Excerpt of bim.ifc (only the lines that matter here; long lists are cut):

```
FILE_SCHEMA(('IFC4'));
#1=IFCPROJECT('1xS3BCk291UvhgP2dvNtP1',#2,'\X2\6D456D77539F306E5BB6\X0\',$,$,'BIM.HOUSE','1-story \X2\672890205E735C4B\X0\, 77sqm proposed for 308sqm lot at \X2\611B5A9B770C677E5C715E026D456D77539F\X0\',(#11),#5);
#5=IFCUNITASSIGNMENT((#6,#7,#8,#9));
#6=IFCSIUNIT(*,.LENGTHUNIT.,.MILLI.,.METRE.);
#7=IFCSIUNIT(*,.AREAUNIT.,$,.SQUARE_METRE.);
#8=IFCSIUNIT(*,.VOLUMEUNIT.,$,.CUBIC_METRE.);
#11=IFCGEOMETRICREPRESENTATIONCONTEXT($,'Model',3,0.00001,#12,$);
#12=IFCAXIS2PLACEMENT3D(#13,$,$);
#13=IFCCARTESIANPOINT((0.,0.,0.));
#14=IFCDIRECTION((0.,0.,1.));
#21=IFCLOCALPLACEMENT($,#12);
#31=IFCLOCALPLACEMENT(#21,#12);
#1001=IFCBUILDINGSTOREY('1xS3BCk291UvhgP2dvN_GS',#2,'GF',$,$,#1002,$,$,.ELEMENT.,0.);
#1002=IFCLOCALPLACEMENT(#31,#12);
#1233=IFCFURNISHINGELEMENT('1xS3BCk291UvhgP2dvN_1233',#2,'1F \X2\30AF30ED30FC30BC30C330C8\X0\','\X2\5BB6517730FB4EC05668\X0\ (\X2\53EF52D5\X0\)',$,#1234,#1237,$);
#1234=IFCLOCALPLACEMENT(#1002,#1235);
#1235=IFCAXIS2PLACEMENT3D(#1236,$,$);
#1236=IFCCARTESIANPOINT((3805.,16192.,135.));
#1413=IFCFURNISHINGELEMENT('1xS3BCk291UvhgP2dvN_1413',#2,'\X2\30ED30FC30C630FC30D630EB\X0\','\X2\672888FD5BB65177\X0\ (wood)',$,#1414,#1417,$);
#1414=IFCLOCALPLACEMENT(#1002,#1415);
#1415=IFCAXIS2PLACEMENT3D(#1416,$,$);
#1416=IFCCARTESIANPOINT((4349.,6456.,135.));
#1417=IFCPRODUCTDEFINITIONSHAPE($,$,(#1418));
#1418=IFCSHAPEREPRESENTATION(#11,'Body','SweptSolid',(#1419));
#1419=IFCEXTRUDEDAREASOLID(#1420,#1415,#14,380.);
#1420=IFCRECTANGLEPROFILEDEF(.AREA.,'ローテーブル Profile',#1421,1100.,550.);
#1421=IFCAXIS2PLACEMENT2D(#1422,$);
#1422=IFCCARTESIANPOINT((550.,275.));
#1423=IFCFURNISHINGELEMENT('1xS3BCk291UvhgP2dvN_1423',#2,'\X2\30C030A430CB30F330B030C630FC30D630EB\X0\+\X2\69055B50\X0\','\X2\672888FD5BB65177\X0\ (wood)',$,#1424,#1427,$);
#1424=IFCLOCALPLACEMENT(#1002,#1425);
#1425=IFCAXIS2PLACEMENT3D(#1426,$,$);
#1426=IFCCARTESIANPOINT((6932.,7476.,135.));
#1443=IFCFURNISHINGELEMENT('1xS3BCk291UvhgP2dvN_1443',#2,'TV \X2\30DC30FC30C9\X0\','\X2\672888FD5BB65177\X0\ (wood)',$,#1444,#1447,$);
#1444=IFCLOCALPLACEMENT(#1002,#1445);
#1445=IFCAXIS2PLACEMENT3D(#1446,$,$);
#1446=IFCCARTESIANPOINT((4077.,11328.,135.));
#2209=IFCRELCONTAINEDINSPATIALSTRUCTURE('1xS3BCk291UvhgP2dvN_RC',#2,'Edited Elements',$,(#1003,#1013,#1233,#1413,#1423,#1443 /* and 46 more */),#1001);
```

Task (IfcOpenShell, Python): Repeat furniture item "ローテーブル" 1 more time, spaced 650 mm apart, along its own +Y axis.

```python
import ifcopenshell
import ifcopenshell.api.geometry
import ifcopenshell.api.root
import ifcopenshell.util.element
import ifcopenshell.util.placement

model = ifcopenshell.open("bim.ifc")


def reuse_history(source, copy):
    """copy_class also copies each property set's owner history, people and application; keep the originals."""
    for rel in copy.IsDefinedBy:
        if rel.is_a("IfcRelDefinesByProperties") and (history := rel.RelatingPropertyDefinition.OwnerHistory):
            rel.RelatingPropertyDefinition.OwnerHistory = source.OwnerHistory
            ifcopenshell.util.element.remove_deep2(model, history)


source = model.by_guid("1xS3BCk291UvhgP2dvN_1413")
base = ifcopenshell.util.placement.get_local_placement(source.ObjectPlacement)
step = base[:3, 1] * 650.0

for i in range(1, 2):
    copy = ifcopenshell.api.root.copy_class(model, product=source)
    copy.Representation = ifcopenshell.util.element.copy_deep(
        model, source.Representation, exclude=["IfcGeometricRepresentationContext", "IfcRepresentationMap"]
    )
    reuse_history(source, copy)
    matrix = base.copy()
    matrix[:3, 3] += i * step
    print("added at", matrix[:3, 3].round(3) + 0.0)
    ifcopenshell.api.geometry.edit_object_placement(model, product=copy, matrix=matrix, is_si=False)

model.write("bim_v2.ifc")
```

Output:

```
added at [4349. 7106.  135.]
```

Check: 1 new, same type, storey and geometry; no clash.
